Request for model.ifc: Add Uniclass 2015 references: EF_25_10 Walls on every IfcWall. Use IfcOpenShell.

First a look at what the model holds.

```python
import ifcopenshell

model = ifcopenshell.open("model.ifc")
print(model.schema)
print("classifications:", [c.Name for c in model.by_type("IfcClassification")])
for ifc_class in ("IfcDoor", "IfcRoof", "IfcStair", "IfcWall", "IfcWindow"):
    print(ifc_class, len(model.by_type(ifc_class)))
```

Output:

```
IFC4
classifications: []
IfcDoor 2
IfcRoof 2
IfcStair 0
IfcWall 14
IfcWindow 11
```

```python
import ifcopenshell
import ifcopenshell.api.classification

model = ifcopenshell.open("model.ifc")

system = ifcopenshell.api.classification.add_classification(model, classification="Uniclass 2015")

codes = {
    "IfcWall": ("EF_25_10", "Walls"),
}
for ifc_class, (code, name) in codes.items():
    products = model.by_type(ifc_class)
    ifcopenshell.api.classification.add_reference(
        model, products=products, classification=system, identification=code, name=name
    )
    print(code, len(products))

model.write("model_edited.ifc")
```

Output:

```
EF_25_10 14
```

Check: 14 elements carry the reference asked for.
